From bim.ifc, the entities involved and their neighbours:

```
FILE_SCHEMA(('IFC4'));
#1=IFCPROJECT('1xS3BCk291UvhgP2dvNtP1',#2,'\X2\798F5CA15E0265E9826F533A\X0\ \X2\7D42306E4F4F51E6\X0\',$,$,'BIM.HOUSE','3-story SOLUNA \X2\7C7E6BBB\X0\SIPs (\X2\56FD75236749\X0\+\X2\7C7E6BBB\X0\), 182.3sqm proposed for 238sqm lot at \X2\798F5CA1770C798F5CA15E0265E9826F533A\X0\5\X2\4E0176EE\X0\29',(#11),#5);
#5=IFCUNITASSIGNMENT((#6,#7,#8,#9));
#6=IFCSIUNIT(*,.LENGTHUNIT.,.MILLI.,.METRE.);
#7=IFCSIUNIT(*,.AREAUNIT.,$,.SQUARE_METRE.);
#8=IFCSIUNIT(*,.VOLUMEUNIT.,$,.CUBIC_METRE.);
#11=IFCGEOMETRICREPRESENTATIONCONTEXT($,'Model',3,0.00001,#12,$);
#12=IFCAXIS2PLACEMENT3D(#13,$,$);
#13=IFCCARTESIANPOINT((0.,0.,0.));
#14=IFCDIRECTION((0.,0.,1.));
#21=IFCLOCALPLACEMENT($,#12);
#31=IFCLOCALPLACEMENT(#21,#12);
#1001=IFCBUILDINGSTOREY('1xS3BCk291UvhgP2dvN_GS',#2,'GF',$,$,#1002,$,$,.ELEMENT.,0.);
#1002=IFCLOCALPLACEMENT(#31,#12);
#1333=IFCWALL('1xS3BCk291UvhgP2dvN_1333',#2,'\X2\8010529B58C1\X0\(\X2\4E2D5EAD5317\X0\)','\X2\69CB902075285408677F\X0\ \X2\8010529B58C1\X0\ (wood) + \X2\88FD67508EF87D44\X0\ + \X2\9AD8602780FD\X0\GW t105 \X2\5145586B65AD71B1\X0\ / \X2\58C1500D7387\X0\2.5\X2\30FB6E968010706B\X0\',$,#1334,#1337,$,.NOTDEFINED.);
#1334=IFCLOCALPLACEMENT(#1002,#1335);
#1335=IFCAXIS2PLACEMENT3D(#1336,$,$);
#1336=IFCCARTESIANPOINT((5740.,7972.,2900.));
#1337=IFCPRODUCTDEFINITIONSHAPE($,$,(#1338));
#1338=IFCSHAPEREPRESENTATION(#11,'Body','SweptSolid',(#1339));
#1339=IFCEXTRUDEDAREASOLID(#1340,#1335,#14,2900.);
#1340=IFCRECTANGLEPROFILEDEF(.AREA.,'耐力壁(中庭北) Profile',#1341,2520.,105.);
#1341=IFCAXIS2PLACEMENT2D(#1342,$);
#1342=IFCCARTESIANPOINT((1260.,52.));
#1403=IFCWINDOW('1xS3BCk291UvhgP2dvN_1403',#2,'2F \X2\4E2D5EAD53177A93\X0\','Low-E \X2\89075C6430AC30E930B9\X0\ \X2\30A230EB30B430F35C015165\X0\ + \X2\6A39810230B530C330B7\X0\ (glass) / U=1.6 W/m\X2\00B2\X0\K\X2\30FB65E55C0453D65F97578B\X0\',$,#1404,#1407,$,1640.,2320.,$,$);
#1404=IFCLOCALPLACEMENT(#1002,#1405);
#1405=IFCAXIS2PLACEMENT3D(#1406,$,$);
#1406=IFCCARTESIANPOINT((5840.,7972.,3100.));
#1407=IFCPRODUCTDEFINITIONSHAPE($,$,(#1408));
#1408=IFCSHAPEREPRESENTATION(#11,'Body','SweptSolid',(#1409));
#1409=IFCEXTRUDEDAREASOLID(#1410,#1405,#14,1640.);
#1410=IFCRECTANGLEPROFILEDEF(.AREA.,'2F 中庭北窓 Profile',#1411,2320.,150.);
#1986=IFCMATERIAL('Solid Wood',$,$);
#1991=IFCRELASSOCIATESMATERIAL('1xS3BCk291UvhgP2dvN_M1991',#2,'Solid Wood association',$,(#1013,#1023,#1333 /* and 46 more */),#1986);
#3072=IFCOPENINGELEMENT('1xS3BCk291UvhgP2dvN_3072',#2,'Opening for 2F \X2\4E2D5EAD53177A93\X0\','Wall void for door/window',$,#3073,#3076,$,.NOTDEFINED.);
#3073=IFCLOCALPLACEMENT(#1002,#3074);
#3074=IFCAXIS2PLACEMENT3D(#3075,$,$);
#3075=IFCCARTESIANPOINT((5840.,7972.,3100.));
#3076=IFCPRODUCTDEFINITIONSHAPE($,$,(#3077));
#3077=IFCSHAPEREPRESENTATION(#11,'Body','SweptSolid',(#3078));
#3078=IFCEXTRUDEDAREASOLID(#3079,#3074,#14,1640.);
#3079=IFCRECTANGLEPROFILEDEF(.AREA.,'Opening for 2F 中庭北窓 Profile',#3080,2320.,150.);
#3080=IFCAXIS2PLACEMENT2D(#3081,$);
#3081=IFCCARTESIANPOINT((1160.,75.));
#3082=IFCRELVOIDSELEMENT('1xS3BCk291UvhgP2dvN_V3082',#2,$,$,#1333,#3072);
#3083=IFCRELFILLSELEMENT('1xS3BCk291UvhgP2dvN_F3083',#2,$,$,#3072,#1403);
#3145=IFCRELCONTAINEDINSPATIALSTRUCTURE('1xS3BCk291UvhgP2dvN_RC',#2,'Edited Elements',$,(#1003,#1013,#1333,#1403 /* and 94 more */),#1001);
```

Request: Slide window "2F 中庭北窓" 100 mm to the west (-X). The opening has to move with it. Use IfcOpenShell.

```python
import ifcopenshell
import ifcopenshell.api.geometry
import ifcopenshell.util.placement
import ifcopenshell.util.unit

model = ifcopenshell.open("bim.ifc")
unit_scale = ifcopenshell.util.unit.calculate_unit_scale(model)

window = model.by_guid("1xS3BCk291UvhgP2dvN_1403")
opening = window.FillsVoids[0].RelatingOpeningElement
wall = opening.VoidsElements[0].RelatingBuildingElement

wall_matrix = ifcopenshell.util.placement.get_local_placement(wall.ObjectPlacement)
shift = wall_matrix[:3, 0] * -0.1 / unit_scale
before = ifcopenshell.util.placement.get_local_placement(window.ObjectPlacement)[:3, 3].copy()

# The window is not placed relative to its opening, so move both.
for product in (opening, window):
    matrix = ifcopenshell.util.placement.get_local_placement(product.ObjectPlacement)
    matrix[:3, 3] += shift
    ifcopenshell.api.geometry.edit_object_placement(model, product=product, matrix=matrix, is_si=False)

after = ifcopenshell.util.placement.get_local_placement(window.ObjectPlacement)[:3, 3]
print("window moved by", (after - before).round(3) + 0.0)

model.write("bim_updated.ifc")
```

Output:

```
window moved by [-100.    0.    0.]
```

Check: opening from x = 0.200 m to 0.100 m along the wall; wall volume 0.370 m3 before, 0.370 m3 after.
